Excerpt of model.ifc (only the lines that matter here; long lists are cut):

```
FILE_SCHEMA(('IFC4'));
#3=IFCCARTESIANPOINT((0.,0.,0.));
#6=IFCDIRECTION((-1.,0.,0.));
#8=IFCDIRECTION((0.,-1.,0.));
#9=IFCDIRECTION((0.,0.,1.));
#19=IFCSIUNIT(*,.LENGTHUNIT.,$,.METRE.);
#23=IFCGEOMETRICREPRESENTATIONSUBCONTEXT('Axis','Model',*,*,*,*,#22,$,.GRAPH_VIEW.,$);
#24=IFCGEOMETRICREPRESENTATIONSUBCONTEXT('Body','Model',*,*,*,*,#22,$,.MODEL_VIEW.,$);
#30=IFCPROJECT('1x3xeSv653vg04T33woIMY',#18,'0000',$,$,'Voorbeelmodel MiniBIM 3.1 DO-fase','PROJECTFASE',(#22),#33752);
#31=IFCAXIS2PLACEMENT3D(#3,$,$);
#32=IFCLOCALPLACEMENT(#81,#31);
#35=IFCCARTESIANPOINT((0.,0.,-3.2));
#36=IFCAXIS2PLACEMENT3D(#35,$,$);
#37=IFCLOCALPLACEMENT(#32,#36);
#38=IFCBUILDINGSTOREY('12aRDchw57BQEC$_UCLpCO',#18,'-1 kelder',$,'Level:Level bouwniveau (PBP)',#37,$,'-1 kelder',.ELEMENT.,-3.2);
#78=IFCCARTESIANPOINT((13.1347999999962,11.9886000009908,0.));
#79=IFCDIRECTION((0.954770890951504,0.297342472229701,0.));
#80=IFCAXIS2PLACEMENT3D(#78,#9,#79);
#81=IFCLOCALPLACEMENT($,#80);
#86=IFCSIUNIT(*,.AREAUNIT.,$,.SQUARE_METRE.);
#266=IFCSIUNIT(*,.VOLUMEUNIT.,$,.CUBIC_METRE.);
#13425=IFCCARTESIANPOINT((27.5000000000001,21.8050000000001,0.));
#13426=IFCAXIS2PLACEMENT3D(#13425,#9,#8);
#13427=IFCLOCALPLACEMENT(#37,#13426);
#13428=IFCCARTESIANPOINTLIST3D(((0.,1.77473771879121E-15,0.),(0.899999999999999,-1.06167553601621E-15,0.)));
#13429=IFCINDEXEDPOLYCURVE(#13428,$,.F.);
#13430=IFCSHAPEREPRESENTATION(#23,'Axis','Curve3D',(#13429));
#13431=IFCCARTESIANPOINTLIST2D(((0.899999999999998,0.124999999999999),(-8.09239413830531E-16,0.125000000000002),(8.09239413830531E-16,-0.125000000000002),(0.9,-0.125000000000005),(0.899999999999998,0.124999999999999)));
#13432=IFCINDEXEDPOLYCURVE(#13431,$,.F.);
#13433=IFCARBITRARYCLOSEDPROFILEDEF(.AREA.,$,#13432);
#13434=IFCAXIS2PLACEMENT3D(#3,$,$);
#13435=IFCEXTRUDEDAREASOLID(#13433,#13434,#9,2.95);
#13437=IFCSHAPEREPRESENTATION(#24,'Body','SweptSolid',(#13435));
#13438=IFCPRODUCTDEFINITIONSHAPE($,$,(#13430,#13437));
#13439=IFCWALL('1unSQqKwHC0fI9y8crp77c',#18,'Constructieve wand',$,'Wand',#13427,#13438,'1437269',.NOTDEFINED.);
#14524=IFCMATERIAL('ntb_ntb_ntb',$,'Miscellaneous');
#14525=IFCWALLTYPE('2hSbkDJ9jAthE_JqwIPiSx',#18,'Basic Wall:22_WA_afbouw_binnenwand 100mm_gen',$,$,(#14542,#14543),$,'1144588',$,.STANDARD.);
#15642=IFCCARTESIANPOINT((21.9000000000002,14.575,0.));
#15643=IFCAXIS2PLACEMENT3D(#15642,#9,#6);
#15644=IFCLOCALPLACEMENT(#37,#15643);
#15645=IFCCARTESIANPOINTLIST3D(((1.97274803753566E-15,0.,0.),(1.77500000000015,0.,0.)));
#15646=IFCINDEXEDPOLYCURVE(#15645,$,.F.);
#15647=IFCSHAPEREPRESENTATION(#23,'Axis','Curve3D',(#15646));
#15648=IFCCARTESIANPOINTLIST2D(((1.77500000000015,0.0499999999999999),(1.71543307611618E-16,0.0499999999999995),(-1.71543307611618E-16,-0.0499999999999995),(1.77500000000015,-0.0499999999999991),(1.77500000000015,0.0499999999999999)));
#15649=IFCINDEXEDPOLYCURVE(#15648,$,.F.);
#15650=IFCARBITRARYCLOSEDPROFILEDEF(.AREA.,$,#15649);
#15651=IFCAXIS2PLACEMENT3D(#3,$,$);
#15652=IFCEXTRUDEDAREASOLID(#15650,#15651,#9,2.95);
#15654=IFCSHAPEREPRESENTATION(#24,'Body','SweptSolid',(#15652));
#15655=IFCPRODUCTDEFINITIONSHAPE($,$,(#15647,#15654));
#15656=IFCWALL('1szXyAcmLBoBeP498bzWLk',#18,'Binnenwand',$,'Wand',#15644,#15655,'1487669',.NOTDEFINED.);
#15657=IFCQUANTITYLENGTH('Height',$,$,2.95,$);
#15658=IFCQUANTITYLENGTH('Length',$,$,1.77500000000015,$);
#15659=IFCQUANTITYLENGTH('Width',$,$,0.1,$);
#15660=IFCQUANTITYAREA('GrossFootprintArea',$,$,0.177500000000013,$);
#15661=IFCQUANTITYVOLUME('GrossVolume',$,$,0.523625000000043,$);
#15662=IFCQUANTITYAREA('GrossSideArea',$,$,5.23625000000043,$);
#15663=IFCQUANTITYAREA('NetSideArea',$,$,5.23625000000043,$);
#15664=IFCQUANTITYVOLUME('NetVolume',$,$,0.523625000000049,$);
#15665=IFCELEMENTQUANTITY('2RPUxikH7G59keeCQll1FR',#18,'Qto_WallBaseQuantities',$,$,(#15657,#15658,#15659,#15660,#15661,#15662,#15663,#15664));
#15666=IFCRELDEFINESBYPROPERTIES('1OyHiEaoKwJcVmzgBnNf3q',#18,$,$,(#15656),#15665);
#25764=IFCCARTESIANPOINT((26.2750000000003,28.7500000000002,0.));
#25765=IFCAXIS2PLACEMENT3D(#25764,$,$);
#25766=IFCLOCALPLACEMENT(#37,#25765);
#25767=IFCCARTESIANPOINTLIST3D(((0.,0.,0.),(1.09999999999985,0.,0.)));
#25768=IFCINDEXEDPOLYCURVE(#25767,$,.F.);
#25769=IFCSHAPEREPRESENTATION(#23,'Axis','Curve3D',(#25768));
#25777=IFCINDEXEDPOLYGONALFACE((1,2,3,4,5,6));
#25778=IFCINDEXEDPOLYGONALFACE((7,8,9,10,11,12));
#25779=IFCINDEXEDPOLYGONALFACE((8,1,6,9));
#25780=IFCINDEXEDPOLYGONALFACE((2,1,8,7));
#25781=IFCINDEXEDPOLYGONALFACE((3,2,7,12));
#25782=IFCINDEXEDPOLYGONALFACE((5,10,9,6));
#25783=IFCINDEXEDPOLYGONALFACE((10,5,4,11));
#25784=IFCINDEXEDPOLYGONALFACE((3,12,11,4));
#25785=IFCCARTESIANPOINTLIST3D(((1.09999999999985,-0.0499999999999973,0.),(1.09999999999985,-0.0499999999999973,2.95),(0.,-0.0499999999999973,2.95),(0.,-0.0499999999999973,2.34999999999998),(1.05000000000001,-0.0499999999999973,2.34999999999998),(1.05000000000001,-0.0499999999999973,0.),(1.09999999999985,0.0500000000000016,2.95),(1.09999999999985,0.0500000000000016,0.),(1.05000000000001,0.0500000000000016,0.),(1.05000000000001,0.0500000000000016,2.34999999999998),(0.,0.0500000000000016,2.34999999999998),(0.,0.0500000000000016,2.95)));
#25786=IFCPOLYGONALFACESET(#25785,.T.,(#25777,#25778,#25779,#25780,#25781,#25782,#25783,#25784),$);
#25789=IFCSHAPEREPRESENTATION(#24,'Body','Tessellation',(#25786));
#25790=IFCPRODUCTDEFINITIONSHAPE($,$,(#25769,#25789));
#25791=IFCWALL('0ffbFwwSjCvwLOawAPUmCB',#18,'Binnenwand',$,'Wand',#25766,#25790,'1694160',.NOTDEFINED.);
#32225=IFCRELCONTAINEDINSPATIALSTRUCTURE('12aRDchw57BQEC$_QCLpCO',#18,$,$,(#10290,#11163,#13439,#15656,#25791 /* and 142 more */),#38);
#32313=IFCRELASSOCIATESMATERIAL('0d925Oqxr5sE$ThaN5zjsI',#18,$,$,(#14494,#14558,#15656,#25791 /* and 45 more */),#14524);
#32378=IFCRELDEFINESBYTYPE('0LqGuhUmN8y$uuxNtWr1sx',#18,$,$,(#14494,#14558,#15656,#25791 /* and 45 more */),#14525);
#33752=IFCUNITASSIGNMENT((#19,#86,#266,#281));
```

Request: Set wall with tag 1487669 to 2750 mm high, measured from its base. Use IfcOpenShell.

```python
import ifcopenshell
import ifcopenshell.api.pset
import ifcopenshell.geom
import ifcopenshell.util.element
import ifcopenshell.util.representation
import ifcopenshell.util.shape
import ifcopenshell.util.unit

model = ifcopenshell.open("model.ifc")
unit_scale = ifcopenshell.util.unit.calculate_unit_scale(model)
area_scale = ifcopenshell.util.unit.calculate_unit_scale(model, "AREAUNIT")
volume_scale = ifcopenshell.util.unit.calculate_unit_scale(model, "VOLUMEUNIT")
settings = ifcopenshell.geom.settings()


def volume(element):
    """Net volume in cubic metres, openings subtracted."""
    shape = ifcopenshell.geom.create_shape(settings, element)
    return ifcopenshell.util.shape.get_volume(shape.geometry)


wall = model.by_id(15656)
before = volume(wall)

body = ifcopenshell.util.representation.get_representation(wall, "Model", "Body")
solid = body.Items[0]
old_height = solid.Depth
solid.Depth = 2.75 / unit_scale
after = volume(wall)
thickness = 0.1  # wall thickness in metres

# Update the stored height, areas and volumes.
qto = model.by_id(ifcopenshell.util.element.get_pset(wall, "Qto_WallBaseQuantities", should_inherit=False)["id"])
ifcopenshell.api.pset.edit_qto(model, qto=qto, properties={
    "Height": solid.Depth,
    "GrossVolume": ifcopenshell.util.element.get_pset(wall, "Qto_WallBaseQuantities", "GrossVolume") * solid.Depth / old_height,
    "GrossSideArea": ifcopenshell.util.element.get_pset(wall, "Qto_WallBaseQuantities", "GrossSideArea") * solid.Depth / old_height,
    "NetSideArea": after / thickness / area_scale,
    "NetVolume": after / volume_scale,
})

print(f"height {old_height:g} -> {solid.Depth:g}, volume {before:.3f} -> {after:.3f} m3")

model.write("model_rev.ifc")
```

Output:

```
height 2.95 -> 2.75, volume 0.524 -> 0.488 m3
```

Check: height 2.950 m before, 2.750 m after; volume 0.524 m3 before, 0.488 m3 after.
